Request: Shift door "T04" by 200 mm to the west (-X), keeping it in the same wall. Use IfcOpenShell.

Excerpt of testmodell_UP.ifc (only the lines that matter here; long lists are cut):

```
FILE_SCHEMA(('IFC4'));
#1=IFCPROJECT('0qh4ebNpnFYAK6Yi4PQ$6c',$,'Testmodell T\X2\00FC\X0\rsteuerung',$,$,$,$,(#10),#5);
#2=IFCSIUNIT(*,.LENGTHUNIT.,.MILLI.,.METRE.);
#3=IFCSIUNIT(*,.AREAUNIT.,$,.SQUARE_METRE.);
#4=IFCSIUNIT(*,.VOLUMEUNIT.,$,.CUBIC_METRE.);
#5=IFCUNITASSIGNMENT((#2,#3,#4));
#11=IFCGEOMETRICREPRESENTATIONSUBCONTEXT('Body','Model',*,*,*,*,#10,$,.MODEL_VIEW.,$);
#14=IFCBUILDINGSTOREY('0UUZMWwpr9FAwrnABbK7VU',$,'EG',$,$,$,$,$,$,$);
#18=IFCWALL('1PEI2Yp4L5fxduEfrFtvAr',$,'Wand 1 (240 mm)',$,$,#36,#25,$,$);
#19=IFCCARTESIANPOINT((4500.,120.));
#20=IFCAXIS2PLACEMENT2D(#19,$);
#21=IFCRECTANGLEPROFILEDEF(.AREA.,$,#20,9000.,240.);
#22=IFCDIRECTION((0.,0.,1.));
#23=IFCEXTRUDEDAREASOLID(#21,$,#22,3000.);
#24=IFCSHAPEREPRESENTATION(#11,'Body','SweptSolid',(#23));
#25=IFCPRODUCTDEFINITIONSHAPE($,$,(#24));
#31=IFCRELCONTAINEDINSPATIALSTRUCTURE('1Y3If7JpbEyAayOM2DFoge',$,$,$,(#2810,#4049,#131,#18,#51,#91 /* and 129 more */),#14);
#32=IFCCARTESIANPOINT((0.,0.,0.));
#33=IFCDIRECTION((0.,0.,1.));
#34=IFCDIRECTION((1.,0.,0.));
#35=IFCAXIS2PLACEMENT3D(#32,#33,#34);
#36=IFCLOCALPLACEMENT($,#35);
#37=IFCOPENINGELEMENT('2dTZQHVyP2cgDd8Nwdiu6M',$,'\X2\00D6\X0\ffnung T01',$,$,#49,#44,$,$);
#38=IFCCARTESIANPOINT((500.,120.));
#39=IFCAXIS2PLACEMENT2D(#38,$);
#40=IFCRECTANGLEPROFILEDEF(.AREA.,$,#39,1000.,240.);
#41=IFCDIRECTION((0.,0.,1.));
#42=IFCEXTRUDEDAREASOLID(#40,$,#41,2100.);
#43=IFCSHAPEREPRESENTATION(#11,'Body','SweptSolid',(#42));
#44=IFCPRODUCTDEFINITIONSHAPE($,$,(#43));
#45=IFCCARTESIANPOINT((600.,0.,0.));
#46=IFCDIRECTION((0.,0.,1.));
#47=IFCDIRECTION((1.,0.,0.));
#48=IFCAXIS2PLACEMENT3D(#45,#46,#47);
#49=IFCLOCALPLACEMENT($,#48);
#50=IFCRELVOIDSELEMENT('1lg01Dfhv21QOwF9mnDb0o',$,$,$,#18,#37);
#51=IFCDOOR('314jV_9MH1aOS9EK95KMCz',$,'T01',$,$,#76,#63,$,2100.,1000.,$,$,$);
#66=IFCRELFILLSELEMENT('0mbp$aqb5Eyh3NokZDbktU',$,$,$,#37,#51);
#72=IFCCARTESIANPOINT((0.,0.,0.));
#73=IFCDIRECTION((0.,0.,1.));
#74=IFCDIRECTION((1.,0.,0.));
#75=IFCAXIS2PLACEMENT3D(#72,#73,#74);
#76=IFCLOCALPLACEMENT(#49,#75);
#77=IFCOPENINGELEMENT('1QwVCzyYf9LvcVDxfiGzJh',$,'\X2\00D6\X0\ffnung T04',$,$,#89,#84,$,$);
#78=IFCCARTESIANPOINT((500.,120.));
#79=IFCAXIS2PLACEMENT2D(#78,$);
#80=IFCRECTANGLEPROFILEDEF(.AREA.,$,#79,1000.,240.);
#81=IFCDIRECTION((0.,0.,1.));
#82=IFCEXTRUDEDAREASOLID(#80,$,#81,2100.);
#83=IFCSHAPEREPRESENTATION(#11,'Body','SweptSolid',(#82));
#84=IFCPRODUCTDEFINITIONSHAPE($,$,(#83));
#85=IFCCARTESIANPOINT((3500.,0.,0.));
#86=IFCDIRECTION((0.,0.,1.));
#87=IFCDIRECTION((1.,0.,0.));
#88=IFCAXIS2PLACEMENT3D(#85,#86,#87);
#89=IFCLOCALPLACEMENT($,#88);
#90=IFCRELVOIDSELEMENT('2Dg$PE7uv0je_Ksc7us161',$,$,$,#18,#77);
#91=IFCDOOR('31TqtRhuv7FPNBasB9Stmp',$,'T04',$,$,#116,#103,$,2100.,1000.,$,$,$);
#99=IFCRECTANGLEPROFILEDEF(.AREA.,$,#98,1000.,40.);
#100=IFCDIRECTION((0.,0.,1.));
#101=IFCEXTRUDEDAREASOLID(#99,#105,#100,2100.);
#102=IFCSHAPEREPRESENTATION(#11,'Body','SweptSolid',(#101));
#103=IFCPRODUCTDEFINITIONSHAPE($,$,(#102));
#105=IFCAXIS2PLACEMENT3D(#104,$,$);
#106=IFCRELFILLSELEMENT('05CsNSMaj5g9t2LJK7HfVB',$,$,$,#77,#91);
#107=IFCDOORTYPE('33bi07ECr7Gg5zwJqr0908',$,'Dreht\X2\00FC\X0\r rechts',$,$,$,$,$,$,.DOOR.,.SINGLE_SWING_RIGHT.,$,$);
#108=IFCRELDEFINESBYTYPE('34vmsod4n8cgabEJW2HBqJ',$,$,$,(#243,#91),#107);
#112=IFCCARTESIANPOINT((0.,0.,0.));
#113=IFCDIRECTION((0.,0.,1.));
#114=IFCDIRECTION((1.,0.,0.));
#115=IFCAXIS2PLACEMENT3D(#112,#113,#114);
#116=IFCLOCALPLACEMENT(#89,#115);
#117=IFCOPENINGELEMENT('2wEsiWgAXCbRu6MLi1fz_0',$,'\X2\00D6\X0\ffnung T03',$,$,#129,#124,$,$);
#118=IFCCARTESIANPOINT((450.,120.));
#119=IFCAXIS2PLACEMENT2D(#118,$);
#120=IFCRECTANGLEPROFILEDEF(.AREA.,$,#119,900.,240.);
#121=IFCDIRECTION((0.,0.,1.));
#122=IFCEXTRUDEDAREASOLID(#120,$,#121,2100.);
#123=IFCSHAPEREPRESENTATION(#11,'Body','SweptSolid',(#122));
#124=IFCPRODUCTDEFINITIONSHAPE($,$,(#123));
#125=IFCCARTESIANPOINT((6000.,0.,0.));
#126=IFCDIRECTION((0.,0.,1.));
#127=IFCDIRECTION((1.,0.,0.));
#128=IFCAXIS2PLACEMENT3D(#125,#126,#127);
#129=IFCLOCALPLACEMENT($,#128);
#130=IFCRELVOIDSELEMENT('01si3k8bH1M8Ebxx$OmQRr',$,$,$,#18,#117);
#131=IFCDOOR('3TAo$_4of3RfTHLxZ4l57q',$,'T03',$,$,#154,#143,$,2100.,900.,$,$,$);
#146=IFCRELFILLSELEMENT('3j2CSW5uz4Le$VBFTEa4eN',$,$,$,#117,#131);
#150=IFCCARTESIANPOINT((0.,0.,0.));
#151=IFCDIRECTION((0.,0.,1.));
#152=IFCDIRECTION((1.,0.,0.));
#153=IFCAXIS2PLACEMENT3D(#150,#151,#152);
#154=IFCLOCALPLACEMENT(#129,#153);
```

```python
import ifcopenshell
import ifcopenshell.api.geometry
import ifcopenshell.util.placement

model = ifcopenshell.open("testmodell_UP.ifc")

door = model.by_guid("31TqtRhuv7FPNBasB9Stmp")
opening = door.FillsVoids[0].RelatingOpeningElement
wall = opening.VoidsElements[0].RelatingBuildingElement

wall_matrix = ifcopenshell.util.placement.get_local_placement(wall.ObjectPlacement)
shift = wall_matrix[:3, 0] * -200.0
before = ifcopenshell.util.placement.get_local_placement(door.ObjectPlacement)[:3, 3].copy()

# The door is placed relative to its opening, so it follows when the opening moves.
matrix = ifcopenshell.util.placement.get_local_placement(opening.ObjectPlacement)
matrix[:3, 3] += shift
ifcopenshell.api.geometry.edit_object_placement(
    model, product=opening, matrix=matrix, is_si=False, should_transform_children=True
)

after = ifcopenshell.util.placement.get_local_placement(door.ObjectPlacement)[:3, 3]
print("door moved by", (after - before).round(3) + 0.0)

model.write("testmodell_UP_edited.ifc")
```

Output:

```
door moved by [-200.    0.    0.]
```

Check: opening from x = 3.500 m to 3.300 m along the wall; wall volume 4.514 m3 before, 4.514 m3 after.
